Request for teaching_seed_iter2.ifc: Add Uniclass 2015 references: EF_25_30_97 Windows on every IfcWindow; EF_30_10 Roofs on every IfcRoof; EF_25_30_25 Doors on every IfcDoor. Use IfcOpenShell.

First a look at what the model holds.

```python
import ifcopenshell

model = ifcopenshell.open("teaching_seed_iter2.ifc")
print(model.schema)
print("classifications:", [c.Name for c in model.by_type("IfcClassification")])
for ifc_class in ("IfcDoor", "IfcRoof", "IfcStair", "IfcWall", "IfcWindow"):
    print(ifc_class, len(model.by_type(ifc_class)))
```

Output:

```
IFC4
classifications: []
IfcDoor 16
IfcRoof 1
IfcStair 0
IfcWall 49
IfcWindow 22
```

```python
import ifcopenshell
import ifcopenshell.api.classification

model = ifcopenshell.open("teaching_seed_iter2.ifc")

system = ifcopenshell.api.classification.add_classification(model, classification="Uniclass 2015")

codes = {
    "IfcWindow": ("EF_25_30_97", "Windows"),
    "IfcRoof": ("EF_30_10", "Roofs"),
    "IfcDoor": ("EF_25_30_25", "Doors"),
}
for ifc_class, (code, name) in codes.items():
    products = model.by_type(ifc_class)
    ifcopenshell.api.classification.add_reference(
        model, products=products, classification=system, identification=code, name=name
    )
    print(code, len(products))

model.write("teaching_seed_iter2_edited.ifc")
```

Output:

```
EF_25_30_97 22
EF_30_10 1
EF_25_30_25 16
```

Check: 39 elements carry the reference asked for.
